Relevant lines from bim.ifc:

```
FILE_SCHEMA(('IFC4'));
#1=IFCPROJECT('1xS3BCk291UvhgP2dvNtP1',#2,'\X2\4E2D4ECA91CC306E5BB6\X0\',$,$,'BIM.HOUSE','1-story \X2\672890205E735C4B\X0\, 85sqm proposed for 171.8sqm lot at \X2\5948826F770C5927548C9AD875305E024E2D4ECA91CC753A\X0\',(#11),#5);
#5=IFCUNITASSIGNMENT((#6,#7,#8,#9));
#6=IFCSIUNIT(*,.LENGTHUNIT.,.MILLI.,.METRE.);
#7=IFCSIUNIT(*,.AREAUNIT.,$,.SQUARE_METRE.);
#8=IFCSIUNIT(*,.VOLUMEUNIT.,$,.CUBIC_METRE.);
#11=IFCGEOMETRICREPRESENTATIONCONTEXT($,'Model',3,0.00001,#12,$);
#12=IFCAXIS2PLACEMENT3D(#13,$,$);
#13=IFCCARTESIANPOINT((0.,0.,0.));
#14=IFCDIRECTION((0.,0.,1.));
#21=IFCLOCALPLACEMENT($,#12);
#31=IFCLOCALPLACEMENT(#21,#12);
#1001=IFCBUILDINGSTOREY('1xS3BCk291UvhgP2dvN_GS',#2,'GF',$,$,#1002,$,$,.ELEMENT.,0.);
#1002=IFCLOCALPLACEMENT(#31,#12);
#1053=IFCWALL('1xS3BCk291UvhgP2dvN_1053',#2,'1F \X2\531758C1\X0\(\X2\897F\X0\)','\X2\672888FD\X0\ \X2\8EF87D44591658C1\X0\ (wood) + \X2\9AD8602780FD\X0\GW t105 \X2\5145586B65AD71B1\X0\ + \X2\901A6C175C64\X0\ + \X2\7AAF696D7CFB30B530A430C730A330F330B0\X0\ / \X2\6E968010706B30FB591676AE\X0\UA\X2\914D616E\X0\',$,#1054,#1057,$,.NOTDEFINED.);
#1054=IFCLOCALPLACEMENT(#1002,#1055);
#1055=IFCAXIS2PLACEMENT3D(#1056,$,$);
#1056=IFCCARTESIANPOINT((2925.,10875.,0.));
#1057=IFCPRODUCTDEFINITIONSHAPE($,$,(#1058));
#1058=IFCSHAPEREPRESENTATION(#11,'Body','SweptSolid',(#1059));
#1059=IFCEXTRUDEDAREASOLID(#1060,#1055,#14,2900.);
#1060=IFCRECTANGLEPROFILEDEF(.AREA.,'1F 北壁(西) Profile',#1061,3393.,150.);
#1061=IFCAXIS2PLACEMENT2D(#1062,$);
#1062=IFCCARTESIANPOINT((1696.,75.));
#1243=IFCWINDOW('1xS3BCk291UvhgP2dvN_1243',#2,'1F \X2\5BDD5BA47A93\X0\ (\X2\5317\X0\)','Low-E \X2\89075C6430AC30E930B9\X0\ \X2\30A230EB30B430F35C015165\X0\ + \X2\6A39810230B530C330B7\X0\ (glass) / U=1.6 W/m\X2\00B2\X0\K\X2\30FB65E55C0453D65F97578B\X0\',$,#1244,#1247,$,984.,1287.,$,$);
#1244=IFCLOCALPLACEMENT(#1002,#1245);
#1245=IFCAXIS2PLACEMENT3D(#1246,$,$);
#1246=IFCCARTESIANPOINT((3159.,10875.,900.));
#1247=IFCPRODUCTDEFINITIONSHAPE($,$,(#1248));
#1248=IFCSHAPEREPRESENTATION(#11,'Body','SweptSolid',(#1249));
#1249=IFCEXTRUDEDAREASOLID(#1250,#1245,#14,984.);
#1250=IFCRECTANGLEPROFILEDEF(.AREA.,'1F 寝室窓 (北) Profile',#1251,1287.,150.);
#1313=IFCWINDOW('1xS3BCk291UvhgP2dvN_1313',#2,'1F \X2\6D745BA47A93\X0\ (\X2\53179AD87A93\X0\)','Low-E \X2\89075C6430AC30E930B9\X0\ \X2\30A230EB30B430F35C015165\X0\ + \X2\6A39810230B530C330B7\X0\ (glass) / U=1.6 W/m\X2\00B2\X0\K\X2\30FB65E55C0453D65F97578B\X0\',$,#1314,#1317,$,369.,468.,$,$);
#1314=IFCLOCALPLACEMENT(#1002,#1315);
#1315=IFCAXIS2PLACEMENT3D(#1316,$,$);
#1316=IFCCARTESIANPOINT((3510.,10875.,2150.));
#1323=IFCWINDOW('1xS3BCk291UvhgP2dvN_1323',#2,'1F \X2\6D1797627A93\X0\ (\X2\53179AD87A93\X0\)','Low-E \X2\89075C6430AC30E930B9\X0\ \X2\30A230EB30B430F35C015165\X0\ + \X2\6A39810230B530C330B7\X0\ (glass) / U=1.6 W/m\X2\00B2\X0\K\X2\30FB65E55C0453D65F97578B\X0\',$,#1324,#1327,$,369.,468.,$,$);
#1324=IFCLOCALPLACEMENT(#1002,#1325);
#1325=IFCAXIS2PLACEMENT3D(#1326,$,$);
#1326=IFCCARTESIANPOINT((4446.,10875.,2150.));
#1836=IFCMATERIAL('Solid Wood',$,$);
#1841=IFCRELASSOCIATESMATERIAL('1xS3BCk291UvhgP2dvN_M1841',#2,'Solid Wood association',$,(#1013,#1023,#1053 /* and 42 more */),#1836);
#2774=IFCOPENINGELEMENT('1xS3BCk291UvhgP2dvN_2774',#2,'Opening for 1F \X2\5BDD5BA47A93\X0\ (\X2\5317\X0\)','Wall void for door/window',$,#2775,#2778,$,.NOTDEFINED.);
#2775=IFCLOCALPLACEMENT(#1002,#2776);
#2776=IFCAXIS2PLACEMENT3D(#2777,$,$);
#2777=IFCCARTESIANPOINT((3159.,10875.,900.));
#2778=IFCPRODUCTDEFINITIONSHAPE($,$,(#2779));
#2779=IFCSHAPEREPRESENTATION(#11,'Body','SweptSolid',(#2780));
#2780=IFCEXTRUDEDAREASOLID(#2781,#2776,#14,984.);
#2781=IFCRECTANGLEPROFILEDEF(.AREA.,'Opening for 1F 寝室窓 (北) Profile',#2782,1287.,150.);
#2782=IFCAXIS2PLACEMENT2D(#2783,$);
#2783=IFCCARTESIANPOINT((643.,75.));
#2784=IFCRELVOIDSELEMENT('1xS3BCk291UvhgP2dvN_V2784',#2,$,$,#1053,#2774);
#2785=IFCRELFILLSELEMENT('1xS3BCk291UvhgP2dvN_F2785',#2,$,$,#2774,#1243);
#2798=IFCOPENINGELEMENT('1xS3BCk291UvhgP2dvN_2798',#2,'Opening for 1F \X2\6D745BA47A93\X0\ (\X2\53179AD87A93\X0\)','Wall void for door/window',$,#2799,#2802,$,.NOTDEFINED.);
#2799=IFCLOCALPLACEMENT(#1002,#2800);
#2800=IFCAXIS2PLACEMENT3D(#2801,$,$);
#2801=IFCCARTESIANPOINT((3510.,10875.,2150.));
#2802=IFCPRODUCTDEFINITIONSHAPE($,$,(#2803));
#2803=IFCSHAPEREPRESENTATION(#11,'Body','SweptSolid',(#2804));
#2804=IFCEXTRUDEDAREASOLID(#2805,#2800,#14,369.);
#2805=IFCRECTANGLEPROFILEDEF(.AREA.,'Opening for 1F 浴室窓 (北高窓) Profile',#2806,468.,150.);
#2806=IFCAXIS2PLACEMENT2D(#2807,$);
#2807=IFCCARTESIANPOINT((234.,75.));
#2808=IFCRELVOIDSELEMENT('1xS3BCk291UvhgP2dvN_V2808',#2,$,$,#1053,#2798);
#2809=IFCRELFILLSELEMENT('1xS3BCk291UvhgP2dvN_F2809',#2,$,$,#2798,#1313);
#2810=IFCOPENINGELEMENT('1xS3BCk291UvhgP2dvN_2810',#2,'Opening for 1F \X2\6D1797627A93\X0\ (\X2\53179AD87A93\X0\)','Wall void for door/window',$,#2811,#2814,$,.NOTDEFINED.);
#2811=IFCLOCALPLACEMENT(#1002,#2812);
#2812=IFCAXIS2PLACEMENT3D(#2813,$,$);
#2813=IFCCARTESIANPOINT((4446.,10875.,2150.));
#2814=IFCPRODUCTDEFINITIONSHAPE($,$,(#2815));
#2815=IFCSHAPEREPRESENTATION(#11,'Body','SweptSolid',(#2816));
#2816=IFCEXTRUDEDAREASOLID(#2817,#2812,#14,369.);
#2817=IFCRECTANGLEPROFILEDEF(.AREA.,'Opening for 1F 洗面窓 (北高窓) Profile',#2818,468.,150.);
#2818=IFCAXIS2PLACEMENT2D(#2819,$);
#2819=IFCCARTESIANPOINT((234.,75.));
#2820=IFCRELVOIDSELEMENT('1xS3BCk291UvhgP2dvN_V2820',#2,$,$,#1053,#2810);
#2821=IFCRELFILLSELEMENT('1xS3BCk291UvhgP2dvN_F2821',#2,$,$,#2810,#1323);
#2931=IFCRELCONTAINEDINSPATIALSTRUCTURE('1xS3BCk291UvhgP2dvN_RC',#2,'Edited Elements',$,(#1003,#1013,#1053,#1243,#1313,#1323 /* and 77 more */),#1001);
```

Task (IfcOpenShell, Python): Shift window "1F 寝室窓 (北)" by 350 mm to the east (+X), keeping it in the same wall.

```python
import ifcopenshell
import ifcopenshell.api.geometry
import ifcopenshell.util.placement
import ifcopenshell.util.unit

model = ifcopenshell.open("bim.ifc")
unit_scale = ifcopenshell.util.unit.calculate_unit_scale(model)

window = model.by_id(1243)
opening = window.FillsVoids[0].RelatingOpeningElement
wall = opening.VoidsElements[0].RelatingBuildingElement

wall_matrix = ifcopenshell.util.placement.get_local_placement(wall.ObjectPlacement)
shift = wall_matrix[:3, 0] * 0.35 / unit_scale
before = ifcopenshell.util.placement.get_local_placement(window.ObjectPlacement)[:3, 3].copy()

# The window is not placed relative to its opening, so move both.
for product in (opening, window):
    matrix = ifcopenshell.util.placement.get_local_placement(product.ObjectPlacement)
    matrix[:3, 3] += shift
    ifcopenshell.api.geometry.edit_object_placement(model, product=product, matrix=matrix, is_si=False)

after = ifcopenshell.util.placement.get_local_placement(window.ObjectPlacement)[:3, 3]
print("window moved by", (after - before).round(3) + 0.0)

model.write("bim_updated.ifc")
```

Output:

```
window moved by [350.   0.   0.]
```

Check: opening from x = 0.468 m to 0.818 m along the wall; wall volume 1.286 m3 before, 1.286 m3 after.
